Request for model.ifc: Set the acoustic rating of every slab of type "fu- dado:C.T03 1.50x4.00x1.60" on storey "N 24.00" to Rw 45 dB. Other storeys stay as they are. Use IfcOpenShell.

First a look at what the model holds.

```python
import ifcopenshell
import ifcopenshell.util.element

model = ifcopenshell.open("model.ifc")
print(model.schema)
storey = next(s for s in model.by_type("IfcBuildingStorey") if s.Name == "N 24.00")
slabs = [e for e in ifcopenshell.util.element.get_decomposition(storey) if e.is_a("IfcSlab")]
seen = {}
for e in slabs:
    element_type = ifcopenshell.util.element.get_type(e)
    key = (element_type.Name if element_type != e and element_type else None, ifcopenshell.util.element.get_pset(e, "Pset_SlabCommon", "AcousticRating"))
    seen[key] = seen.get(key, 0) + 1
for (name, value), count in sorted(seen.items(), key=str):
    print(count, "x", name, "|", value)
```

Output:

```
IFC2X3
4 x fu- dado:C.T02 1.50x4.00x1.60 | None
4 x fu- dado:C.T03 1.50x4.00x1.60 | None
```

```python
import ifcopenshell
import ifcopenshell.api.pset
import ifcopenshell.util.element

model = ifcopenshell.open("model.ifc")

storey = next(s for s in model.by_type("IfcBuildingStorey") if s.Name == "N 24.00")
slabs = [e for e in ifcopenshell.util.element.get_decomposition(storey) if e.is_a("IfcSlab")]

count = 0
for e in slabs:
    element_type = ifcopenshell.util.element.get_type(e)
    if element_type in (None, e) or element_type.Name != "fu- dado:C.T03 1.50x4.00x1.60":
        continue
    # add_pset returns the element's existing set when there is one.
    pset = ifcopenshell.api.pset.add_pset(model, product=e, name="Pset_SlabCommon")
    ifcopenshell.api.pset.edit_pset(model, pset=pset, properties={"AcousticRating": "Rw 45 dB"})
    count += 1

print(count, "slabs updated")

model.write("model_updated.ifc")
```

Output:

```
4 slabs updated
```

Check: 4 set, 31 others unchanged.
